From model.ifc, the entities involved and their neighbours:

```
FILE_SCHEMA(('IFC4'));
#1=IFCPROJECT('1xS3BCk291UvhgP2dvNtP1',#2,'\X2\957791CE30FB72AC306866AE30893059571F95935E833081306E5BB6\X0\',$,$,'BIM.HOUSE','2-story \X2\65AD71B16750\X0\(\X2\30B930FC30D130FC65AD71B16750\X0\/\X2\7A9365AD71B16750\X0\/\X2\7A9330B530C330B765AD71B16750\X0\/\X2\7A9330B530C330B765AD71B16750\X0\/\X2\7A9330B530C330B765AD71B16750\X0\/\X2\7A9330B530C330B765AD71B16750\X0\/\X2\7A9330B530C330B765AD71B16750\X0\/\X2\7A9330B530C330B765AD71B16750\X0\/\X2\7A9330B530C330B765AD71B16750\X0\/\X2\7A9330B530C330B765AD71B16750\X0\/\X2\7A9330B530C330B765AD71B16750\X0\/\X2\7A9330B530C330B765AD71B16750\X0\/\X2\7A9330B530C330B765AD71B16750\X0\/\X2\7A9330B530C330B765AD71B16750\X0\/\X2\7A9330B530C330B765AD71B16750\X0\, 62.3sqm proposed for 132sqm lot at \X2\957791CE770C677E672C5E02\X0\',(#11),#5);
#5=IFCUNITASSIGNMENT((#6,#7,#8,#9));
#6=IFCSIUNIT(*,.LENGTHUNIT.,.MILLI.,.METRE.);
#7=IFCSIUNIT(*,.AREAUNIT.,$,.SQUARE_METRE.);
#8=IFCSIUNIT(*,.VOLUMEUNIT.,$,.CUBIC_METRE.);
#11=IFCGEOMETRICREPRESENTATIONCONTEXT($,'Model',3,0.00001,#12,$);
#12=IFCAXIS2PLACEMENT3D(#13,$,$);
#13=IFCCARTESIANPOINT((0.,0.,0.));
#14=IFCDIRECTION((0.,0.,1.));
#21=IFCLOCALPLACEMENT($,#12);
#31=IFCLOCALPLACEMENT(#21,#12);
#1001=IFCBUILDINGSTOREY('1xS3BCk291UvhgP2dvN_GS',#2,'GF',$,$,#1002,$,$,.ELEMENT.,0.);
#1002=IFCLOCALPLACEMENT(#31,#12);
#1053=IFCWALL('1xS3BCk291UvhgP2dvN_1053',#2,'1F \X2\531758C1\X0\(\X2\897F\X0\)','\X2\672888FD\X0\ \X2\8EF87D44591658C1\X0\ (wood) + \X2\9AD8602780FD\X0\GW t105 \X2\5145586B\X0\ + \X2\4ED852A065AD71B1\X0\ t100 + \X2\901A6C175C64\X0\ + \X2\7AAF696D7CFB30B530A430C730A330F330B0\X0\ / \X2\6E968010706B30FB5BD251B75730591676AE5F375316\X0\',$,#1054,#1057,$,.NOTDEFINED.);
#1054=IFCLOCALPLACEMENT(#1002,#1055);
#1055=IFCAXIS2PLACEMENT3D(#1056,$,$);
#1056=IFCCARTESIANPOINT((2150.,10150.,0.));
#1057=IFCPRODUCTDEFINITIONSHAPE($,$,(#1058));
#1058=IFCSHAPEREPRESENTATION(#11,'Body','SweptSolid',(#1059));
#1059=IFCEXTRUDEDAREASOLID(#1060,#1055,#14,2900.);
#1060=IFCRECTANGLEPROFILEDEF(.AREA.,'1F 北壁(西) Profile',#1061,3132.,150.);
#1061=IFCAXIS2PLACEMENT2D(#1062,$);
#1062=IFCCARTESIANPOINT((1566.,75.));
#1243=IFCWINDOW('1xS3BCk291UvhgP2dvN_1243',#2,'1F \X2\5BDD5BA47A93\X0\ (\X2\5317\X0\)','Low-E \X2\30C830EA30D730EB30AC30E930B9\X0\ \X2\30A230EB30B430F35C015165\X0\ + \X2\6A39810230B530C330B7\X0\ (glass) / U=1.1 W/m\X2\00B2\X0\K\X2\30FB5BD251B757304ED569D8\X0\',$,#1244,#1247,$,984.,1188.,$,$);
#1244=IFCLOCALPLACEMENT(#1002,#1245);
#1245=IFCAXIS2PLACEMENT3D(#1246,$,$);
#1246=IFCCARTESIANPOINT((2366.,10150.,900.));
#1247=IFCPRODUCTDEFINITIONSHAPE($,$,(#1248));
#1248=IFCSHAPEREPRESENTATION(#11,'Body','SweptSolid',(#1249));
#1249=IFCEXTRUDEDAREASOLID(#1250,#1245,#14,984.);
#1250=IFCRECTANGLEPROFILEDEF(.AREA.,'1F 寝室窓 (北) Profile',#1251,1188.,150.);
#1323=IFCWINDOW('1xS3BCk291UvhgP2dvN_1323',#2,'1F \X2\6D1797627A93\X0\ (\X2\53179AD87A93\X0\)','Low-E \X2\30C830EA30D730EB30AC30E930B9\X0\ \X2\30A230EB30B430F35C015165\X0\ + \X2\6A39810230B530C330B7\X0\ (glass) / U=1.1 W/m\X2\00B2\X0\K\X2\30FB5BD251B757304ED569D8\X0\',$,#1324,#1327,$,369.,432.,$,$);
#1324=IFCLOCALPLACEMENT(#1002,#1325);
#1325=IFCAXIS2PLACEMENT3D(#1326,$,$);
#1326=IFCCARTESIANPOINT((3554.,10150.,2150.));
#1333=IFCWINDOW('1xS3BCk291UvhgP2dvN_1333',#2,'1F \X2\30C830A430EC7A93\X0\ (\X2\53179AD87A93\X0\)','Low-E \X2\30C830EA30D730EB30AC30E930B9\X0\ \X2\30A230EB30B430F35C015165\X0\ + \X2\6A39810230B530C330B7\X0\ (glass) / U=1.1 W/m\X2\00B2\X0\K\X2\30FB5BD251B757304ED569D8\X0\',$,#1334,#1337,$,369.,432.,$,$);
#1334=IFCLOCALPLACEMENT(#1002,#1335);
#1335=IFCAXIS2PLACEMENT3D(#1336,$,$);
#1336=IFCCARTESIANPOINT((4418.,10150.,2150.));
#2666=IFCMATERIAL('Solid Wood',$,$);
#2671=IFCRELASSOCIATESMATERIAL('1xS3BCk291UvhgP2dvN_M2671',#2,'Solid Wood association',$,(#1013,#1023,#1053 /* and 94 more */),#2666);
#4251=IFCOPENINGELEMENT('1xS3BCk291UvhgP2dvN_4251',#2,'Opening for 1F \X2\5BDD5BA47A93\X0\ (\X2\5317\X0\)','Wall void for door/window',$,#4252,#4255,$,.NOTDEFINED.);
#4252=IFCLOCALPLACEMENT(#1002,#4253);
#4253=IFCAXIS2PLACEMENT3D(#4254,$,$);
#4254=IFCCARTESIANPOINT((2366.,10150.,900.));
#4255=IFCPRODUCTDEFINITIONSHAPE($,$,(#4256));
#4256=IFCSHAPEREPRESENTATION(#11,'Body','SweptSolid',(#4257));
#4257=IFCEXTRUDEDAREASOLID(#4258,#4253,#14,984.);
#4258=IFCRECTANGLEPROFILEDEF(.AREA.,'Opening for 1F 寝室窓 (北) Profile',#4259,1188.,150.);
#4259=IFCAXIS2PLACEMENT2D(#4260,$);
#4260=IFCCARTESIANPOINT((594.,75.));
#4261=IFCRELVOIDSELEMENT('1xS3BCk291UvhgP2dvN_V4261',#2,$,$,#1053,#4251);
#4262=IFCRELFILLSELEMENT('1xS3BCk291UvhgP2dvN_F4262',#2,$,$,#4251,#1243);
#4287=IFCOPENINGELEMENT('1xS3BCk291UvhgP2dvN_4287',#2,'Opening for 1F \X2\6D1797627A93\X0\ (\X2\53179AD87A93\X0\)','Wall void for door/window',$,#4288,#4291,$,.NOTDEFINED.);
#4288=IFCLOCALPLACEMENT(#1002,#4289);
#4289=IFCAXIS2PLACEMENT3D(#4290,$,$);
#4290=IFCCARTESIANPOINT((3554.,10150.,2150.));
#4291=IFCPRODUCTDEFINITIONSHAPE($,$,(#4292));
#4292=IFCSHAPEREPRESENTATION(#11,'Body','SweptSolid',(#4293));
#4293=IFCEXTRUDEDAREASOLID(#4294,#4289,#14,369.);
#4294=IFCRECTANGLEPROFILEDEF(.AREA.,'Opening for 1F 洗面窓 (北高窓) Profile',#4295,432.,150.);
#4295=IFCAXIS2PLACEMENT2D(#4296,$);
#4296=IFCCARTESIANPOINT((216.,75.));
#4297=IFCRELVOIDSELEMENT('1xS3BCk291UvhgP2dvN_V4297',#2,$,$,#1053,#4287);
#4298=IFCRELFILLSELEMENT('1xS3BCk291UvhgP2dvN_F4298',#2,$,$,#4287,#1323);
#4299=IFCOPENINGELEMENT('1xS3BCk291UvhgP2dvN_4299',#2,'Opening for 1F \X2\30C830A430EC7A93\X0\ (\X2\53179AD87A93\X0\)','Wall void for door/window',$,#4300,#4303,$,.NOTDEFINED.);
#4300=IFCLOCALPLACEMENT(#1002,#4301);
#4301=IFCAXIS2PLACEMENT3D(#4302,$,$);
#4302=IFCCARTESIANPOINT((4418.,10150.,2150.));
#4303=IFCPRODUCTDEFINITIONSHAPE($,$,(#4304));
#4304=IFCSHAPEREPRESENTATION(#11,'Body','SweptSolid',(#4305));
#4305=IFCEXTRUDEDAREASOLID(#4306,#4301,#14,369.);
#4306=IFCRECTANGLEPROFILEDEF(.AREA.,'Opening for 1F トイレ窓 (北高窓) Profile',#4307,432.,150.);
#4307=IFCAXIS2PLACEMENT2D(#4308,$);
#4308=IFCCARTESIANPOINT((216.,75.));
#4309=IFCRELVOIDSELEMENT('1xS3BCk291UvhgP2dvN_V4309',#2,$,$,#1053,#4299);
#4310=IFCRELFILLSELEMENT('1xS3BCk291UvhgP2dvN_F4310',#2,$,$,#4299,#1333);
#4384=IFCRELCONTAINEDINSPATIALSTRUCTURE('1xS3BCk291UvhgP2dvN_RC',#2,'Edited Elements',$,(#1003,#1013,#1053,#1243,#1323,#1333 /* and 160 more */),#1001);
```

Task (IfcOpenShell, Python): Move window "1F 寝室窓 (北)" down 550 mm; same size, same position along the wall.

```python
import numpy as np
import ifcopenshell
import ifcopenshell.api.geometry
import ifcopenshell.util.placement
import ifcopenshell.util.unit

model = ifcopenshell.open("model.ifc")
unit_scale = ifcopenshell.util.unit.calculate_unit_scale(model)

window = model.by_guid("1xS3BCk291UvhgP2dvN_1243")
opening = window.FillsVoids[0].RelatingOpeningElement
dz = -0.55 / unit_scale

shift = np.array([0.0, 0.0, dz])
# The window is not placed relative to its opening, so move both.
for product in (opening, window):
    matrix = ifcopenshell.util.placement.get_local_placement(product.ObjectPlacement)
    matrix[:3, 3] += shift
    ifcopenshell.api.geometry.edit_object_placement(model, product=product, matrix=matrix, is_si=False)

print(f"moved by {dz * unit_scale:+.3f} m")

model.write("model-out.ifc")
```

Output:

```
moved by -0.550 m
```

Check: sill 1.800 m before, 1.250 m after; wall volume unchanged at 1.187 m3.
